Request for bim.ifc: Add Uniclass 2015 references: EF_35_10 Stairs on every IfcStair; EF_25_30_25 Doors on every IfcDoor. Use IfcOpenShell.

First a look at what the model holds.

```python
import ifcopenshell

model = ifcopenshell.open("bim.ifc")
print(model.schema)
print("classifications:", [c.Name for c in model.by_type("IfcClassification")])
for ifc_class in ("IfcDoor", "IfcRoof", "IfcStair", "IfcWall", "IfcWindow"):
    print(ifc_class, len(model.by_type(ifc_class)))
```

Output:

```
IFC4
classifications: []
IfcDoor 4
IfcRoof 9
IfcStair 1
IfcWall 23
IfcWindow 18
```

```python
import ifcopenshell
import ifcopenshell.api.classification

model = ifcopenshell.open("bim.ifc")

system = ifcopenshell.api.classification.add_classification(model, classification="Uniclass 2015")

codes = {
    "IfcStair": ("EF_35_10", "Stairs"),
    "IfcDoor": ("EF_25_30_25", "Doors"),
}
for ifc_class, (code, name) in codes.items():
    products = model.by_type(ifc_class)
    ifcopenshell.api.classification.add_reference(
        model, products=products, classification=system, identification=code, name=name
    )
    print(code, len(products))

model.write("bim_rev.ifc")
```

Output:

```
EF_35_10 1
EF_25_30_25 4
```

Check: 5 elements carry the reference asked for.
